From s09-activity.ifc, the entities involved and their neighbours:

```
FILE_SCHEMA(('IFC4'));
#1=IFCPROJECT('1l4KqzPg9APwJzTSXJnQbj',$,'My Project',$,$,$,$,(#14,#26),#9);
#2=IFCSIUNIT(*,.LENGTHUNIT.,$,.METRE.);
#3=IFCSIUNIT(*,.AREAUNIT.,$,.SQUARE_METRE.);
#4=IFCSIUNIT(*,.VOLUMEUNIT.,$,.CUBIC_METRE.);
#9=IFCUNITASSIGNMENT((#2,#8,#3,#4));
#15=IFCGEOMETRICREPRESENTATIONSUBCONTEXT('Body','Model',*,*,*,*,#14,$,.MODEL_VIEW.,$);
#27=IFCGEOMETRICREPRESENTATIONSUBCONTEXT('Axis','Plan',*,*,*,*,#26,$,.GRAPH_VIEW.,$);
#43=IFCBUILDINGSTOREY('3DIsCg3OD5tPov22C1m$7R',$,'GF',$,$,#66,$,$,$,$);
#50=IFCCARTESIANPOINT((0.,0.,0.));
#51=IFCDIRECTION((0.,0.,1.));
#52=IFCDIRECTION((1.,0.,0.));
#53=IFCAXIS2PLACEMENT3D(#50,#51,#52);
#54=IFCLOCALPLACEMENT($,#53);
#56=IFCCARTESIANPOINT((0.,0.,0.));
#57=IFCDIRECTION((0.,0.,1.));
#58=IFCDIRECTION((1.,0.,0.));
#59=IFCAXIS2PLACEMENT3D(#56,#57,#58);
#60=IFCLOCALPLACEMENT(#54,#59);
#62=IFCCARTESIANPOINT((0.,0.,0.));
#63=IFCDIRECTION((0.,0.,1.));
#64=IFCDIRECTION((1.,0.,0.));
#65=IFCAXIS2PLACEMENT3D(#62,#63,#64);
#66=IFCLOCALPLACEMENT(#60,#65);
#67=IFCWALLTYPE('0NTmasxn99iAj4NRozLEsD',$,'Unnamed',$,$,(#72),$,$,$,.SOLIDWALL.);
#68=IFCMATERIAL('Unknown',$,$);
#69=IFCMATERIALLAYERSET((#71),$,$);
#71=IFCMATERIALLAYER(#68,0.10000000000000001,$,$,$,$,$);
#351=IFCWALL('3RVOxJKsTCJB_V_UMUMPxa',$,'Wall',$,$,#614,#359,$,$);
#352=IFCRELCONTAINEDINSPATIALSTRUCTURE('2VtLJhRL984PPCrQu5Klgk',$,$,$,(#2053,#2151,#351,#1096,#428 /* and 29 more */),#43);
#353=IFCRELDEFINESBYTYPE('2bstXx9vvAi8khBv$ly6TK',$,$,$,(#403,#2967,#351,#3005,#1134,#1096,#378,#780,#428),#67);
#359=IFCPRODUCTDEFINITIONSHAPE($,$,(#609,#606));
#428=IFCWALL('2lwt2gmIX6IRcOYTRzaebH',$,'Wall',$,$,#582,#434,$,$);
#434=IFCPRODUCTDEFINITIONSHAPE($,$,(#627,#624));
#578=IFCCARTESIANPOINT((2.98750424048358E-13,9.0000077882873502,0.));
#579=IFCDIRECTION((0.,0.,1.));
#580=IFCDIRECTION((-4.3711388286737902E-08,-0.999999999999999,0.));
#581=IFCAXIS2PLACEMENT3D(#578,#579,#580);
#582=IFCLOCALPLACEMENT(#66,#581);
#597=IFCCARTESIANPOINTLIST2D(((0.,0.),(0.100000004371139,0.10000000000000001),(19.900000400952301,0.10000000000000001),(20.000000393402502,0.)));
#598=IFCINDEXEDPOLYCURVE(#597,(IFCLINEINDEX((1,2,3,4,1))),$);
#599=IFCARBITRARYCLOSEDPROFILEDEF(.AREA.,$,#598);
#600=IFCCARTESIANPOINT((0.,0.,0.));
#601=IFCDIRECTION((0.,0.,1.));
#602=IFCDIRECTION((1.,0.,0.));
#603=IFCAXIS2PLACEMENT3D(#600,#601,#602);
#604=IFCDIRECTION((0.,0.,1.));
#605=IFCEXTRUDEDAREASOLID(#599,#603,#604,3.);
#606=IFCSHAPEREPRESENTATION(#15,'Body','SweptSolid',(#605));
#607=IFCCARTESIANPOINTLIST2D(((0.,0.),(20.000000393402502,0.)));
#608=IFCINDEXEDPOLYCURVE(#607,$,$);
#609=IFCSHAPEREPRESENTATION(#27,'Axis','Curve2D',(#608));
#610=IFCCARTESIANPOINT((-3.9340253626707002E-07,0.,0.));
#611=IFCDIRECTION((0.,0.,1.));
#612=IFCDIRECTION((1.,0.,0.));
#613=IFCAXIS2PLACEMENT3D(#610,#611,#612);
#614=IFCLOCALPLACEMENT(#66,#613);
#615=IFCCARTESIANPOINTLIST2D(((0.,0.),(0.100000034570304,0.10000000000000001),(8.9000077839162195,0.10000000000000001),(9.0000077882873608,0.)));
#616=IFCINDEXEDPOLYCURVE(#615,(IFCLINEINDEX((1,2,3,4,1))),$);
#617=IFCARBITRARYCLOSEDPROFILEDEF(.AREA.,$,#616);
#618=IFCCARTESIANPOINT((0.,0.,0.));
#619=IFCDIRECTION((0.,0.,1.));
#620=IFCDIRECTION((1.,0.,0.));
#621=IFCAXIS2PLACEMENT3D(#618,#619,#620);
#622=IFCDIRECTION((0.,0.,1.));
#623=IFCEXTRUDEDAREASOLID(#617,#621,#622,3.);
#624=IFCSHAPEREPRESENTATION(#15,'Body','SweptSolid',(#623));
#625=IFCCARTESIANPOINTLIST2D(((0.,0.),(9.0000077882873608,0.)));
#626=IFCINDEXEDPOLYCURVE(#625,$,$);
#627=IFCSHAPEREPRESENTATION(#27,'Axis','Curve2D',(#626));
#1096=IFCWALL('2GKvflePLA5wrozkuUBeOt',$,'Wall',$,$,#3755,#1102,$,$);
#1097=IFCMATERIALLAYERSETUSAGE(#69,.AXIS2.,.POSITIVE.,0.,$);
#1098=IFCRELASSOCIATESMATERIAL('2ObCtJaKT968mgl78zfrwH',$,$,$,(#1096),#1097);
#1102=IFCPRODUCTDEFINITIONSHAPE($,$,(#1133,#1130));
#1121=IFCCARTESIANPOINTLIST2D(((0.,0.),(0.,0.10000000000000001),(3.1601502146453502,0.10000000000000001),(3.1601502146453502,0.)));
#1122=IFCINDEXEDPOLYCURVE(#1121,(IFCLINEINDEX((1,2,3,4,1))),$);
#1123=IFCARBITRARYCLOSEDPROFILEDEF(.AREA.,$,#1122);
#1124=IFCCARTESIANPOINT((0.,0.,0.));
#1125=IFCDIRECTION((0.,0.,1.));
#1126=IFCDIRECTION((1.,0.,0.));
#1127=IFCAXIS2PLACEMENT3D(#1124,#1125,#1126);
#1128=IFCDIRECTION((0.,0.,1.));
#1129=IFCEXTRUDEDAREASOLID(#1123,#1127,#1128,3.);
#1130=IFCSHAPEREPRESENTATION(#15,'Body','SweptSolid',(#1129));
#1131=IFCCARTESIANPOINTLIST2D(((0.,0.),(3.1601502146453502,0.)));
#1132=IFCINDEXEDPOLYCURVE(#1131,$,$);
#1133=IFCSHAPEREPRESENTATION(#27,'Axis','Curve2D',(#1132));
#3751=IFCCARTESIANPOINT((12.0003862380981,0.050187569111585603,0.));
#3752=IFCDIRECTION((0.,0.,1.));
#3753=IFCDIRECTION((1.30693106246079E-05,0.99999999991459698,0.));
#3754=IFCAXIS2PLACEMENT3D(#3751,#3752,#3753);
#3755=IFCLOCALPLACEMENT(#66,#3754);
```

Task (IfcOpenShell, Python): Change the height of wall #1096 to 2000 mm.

```python
import ifcopenshell
import ifcopenshell.geom
import ifcopenshell.util.representation
import ifcopenshell.util.shape
import ifcopenshell.util.unit

model = ifcopenshell.open("s09-activity.ifc")
unit_scale = ifcopenshell.util.unit.calculate_unit_scale(model)
settings = ifcopenshell.geom.settings()


def volume(element):
    """Net volume in cubic metres, openings subtracted."""
    shape = ifcopenshell.geom.create_shape(settings, element)
    return ifcopenshell.util.shape.get_volume(shape.geometry)


wall = model.by_id(1096)
before = volume(wall)

body = ifcopenshell.util.representation.get_representation(wall, "Model", "Body")
solid = body.Items[0]
old_height = solid.Depth
solid.Depth = 2 / unit_scale
after = volume(wall)

print(f"height {old_height:g} -> {solid.Depth:g}, volume {before:.3f} -> {after:.3f} m3")

model.write("s09-activity_v2.ifc")
```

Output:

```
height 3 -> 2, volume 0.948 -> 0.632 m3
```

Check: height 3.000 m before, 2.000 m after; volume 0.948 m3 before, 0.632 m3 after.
